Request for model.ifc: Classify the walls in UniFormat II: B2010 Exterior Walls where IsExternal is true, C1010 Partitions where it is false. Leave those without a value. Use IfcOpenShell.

First a look at what the model holds.

```python
import ifcopenshell
import ifcopenshell.util.element

model = ifcopenshell.open("model.ifc")
print(model.schema)
print("classifications:", [c.Name for c in model.by_type("IfcClassification")])
values = [ifcopenshell.util.element.get_pset(e, "Pset_WallCommon", "IsExternal") for e in model.by_type("IfcWall")]
for value in (True, False, None):
    print("IsExternal", value, values.count(value))
```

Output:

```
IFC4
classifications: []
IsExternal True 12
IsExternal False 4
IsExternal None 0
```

```python
import ifcopenshell
import ifcopenshell.api.classification
import ifcopenshell.util.element

model = ifcopenshell.open("model.ifc")

system = ifcopenshell.api.classification.add_classification(model, classification="UniFormat II")

walls = model.by_type("IfcWall")
external = {e: ifcopenshell.util.element.get_pset(e, "Pset_WallCommon", "IsExternal") for e in walls}
for flag, code, name in ((True, "B2010", "Exterior Walls"), (False, "C1010", "Partitions")):
    products = [e for e in walls if external[e] is flag]
    ifcopenshell.api.classification.add_reference(
        model, products=products, classification=system, identification=code, name=name
    )
    print(code, len(products))

model.write("model_updated.ifc")
```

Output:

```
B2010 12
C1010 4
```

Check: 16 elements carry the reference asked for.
